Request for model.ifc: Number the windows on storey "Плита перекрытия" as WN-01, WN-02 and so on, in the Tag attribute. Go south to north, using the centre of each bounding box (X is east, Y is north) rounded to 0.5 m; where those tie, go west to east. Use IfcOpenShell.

First a look at what the model holds.

```python
import ifcopenshell
import ifcopenshell.util.element
import ifcopenshell.util.placement

model = ifcopenshell.open("model.ifc")
print(model.schema)
storey = next(s for s in model.by_type("IfcBuildingStorey") if s.Name == "Плита перекрытия")
windows = [e for e in ifcopenshell.util.element.get_decomposition(storey) if e.is_a("IfcWindow")]
for e in sorted(windows, key=lambda e: e.id()):
    origin = ifcopenshell.util.placement.get_local_placement(e.ObjectPlacement)[:3, 3]
    print(e.id(), e.Tag, e.Name, origin.round(2) + 0.0, sep=" | ")
```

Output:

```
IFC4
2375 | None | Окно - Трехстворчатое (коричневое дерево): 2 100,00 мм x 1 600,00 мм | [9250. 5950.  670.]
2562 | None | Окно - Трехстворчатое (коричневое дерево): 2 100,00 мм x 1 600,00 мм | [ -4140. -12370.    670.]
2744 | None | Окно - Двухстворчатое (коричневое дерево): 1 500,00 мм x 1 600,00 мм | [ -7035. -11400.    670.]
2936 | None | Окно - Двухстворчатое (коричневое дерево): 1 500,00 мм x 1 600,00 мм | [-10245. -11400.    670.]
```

```python
import ifcopenshell
import ifcopenshell.geom
import ifcopenshell.util.element
import ifcopenshell.util.shape

model = ifcopenshell.open("model.ifc")
settings = ifcopenshell.geom.settings()
settings.set("use-world-coords", True)


def centre(element):
    shape = ifcopenshell.geom.create_shape(settings, element)
    return ifcopenshell.util.shape.get_bbox_centroid(shape.geometry)


storey = next(s for s in model.by_type("IfcBuildingStorey") if s.Name == "Плита перекрытия")
windows = [e for e in ifcopenshell.util.element.get_decomposition(storey) if e.is_a("IfcWindow")]

# Insertion points can sit at a corner or the storey origin, so sort by the geometry (in metres).
centres = {e: centre(e) for e in windows}
windows.sort(key=lambda e: (round(centres[e][1] / 0.5), centres[e][0]))

for i, e in enumerate(windows, start=1):
    number = f"WN-{i:02d}"
    e.Tag = number
    print(e.id(), number)

model.write("model-out.ifc")
```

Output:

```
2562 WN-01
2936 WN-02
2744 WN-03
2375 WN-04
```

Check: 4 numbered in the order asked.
